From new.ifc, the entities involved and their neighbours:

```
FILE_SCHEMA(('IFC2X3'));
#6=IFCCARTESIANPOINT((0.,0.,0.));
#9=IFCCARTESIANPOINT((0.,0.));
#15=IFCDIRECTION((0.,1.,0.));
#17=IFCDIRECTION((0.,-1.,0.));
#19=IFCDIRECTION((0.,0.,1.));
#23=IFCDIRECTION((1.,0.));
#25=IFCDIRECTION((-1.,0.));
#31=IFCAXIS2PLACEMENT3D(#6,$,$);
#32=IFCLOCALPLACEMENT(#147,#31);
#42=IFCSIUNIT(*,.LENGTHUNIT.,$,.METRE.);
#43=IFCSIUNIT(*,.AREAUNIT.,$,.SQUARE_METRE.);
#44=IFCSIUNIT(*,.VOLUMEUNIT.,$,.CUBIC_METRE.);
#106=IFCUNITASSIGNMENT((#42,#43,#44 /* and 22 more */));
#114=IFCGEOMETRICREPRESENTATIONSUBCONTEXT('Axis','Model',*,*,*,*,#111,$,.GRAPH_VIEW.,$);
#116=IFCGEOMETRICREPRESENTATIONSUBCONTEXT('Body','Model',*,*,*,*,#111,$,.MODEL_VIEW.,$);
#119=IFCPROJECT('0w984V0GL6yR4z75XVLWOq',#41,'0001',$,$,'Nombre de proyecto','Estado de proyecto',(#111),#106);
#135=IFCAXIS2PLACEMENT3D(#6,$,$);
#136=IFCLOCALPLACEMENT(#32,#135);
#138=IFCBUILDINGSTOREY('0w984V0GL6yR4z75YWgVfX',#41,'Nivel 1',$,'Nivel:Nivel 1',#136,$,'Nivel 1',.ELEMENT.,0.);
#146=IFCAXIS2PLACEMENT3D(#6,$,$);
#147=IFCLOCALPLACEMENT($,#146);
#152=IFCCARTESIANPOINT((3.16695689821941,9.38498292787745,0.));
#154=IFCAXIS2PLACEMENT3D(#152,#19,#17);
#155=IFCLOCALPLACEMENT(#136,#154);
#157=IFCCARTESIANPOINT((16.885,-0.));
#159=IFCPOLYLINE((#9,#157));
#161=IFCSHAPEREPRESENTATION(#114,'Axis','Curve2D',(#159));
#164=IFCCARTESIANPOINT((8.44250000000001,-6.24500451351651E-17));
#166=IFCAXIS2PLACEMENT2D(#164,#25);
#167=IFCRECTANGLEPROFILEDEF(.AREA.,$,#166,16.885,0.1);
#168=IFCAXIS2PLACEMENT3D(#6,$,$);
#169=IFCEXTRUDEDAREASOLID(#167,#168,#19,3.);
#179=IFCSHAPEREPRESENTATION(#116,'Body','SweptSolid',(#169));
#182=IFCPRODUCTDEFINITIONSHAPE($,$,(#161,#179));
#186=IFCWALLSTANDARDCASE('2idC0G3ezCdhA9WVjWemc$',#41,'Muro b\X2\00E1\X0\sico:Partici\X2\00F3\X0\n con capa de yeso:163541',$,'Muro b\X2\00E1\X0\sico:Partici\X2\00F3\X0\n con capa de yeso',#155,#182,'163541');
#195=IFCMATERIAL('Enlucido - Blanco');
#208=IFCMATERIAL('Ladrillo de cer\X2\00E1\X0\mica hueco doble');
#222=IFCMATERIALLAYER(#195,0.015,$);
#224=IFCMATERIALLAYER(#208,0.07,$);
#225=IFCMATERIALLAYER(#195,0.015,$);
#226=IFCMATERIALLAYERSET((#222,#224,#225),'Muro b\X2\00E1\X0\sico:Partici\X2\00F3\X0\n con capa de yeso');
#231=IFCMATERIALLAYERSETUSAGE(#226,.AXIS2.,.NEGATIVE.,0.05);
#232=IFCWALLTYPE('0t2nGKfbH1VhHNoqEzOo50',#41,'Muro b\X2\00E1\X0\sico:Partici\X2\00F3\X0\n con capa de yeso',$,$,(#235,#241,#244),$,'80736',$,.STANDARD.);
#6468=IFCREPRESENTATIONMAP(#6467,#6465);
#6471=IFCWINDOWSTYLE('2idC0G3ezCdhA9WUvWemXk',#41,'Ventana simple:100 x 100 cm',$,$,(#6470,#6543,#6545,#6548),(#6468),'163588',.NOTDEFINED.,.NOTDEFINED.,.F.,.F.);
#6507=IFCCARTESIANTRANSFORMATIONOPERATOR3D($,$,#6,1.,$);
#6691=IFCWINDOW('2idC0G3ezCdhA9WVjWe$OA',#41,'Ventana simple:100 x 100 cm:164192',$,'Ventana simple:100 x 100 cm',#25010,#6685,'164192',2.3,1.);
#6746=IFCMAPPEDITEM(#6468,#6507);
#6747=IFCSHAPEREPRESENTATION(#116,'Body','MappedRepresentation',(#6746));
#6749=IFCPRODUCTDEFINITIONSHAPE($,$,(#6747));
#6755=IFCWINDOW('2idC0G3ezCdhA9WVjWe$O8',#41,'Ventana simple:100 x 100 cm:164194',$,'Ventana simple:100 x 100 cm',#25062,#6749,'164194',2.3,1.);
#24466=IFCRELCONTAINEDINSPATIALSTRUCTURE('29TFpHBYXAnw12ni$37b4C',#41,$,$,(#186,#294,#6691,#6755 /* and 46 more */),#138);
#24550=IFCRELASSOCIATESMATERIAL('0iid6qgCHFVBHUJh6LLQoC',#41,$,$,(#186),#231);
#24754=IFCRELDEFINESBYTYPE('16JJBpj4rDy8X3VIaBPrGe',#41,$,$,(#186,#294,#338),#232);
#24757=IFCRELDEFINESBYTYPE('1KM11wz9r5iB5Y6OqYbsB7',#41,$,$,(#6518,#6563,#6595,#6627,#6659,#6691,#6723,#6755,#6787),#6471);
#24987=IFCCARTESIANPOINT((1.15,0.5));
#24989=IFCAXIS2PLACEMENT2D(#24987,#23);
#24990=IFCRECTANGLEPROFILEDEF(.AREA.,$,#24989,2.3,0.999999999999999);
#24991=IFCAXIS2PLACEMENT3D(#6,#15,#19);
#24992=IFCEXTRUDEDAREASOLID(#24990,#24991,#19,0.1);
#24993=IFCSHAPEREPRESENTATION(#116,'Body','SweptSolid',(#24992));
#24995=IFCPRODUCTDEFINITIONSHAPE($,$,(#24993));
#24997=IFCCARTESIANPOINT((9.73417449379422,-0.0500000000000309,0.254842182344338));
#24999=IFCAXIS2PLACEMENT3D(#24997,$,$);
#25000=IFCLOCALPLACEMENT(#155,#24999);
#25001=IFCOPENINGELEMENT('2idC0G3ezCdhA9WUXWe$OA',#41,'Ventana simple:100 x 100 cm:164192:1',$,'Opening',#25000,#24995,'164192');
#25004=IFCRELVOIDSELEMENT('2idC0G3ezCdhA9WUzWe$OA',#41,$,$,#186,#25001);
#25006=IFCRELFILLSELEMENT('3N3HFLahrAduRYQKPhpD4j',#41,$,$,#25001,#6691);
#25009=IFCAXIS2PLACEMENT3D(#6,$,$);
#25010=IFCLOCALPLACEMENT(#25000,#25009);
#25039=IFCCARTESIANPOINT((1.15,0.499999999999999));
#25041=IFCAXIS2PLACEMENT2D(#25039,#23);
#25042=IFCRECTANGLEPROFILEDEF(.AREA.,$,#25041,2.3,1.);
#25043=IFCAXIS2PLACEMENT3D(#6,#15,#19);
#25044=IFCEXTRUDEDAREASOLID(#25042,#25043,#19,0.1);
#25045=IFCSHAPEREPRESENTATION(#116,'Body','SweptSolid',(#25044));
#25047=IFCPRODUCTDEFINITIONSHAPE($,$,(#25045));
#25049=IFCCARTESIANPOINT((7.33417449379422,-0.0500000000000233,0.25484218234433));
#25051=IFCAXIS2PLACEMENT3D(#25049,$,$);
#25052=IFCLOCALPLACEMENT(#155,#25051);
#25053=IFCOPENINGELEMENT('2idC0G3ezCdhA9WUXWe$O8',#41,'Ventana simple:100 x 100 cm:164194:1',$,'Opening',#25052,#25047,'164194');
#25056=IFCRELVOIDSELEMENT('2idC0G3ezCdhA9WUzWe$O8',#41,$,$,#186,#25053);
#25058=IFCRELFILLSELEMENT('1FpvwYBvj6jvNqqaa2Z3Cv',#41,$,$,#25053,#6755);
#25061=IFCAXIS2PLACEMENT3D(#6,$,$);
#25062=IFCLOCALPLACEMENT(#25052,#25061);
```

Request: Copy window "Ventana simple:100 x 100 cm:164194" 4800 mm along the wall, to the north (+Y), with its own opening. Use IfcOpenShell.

```python
import ifcopenshell
import ifcopenshell.api.feature
import ifcopenshell.api.geometry
import ifcopenshell.api.root
import ifcopenshell.geom
import ifcopenshell.util.element
import ifcopenshell.util.placement
import ifcopenshell.util.shape

model = ifcopenshell.open("new.ifc")
settings = ifcopenshell.geom.settings()


def volume(element):
    """Net volume in cubic metres, openings subtracted."""
    shape = ifcopenshell.geom.create_shape(settings, element)
    return ifcopenshell.util.shape.get_volume(shape.geometry)


def reuse_history(source, copy):
    """copy_class also copies each property set's owner history, people and application; keep the originals."""
    for rel in copy.IsDefinedBy:
        if rel.is_a("IfcRelDefinesByProperties") and (history := rel.RelatingPropertyDefinition.OwnerHistory):
            rel.RelatingPropertyDefinition.OwnerHistory = source.OwnerHistory
            ifcopenshell.util.element.remove_deep2(model, history)


window = model.by_guid("2idC0G3ezCdhA9WVjWe$O8")
opening = window.FillsVoids[0].RelatingOpeningElement
wall = opening.VoidsElements[0].RelatingBuildingElement
before = volume(wall)
shift = ifcopenshell.util.placement.get_local_placement(wall.ObjectPlacement)[:3, 0] * -4.8

# copy_class copies the void relationship, type, container and properties, but no geometry.
new_opening = ifcopenshell.api.root.copy_class(model, product=opening)
new_opening.Representation = ifcopenshell.util.element.copy_deep(
    model, opening.Representation, exclude=["IfcGeometricRepresentationContext", "IfcRepresentationMap"]
)
new_opening.Name = "Ventana simple:100 x 100 cm"
new_opening.Tag = None
new_window = ifcopenshell.api.root.copy_class(model, product=window)
new_window.Representation = ifcopenshell.util.element.copy_deep(
    model, window.Representation, exclude=["IfcGeometricRepresentationContext", "IfcRepresentationMap"]
)
new_window.Name = "Ventana simple:100 x 100 cm"
new_window.Tag = None
reuse_history(window, new_window)
fills = ifcopenshell.api.feature.add_filling(model, opening=new_opening, element=new_window)
fills.OwnerHistory = new_window.OwnerHistory  # required in IFC2X3

for old, new in ((opening, new_opening), (window, new_window)):
    matrix = ifcopenshell.util.placement.get_local_placement(old.ObjectPlacement)
    matrix[:3, 3] += shift
    ifcopenshell.api.geometry.edit_object_placement(model, product=new, matrix=matrix, is_si=False)

after = volume(wall)

print(f"wall volume {before:.3f} -> {after:.3f} m3")

model.write("new_edited.ifc")
```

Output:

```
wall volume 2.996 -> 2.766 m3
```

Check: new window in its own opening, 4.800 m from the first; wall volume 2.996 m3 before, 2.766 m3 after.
